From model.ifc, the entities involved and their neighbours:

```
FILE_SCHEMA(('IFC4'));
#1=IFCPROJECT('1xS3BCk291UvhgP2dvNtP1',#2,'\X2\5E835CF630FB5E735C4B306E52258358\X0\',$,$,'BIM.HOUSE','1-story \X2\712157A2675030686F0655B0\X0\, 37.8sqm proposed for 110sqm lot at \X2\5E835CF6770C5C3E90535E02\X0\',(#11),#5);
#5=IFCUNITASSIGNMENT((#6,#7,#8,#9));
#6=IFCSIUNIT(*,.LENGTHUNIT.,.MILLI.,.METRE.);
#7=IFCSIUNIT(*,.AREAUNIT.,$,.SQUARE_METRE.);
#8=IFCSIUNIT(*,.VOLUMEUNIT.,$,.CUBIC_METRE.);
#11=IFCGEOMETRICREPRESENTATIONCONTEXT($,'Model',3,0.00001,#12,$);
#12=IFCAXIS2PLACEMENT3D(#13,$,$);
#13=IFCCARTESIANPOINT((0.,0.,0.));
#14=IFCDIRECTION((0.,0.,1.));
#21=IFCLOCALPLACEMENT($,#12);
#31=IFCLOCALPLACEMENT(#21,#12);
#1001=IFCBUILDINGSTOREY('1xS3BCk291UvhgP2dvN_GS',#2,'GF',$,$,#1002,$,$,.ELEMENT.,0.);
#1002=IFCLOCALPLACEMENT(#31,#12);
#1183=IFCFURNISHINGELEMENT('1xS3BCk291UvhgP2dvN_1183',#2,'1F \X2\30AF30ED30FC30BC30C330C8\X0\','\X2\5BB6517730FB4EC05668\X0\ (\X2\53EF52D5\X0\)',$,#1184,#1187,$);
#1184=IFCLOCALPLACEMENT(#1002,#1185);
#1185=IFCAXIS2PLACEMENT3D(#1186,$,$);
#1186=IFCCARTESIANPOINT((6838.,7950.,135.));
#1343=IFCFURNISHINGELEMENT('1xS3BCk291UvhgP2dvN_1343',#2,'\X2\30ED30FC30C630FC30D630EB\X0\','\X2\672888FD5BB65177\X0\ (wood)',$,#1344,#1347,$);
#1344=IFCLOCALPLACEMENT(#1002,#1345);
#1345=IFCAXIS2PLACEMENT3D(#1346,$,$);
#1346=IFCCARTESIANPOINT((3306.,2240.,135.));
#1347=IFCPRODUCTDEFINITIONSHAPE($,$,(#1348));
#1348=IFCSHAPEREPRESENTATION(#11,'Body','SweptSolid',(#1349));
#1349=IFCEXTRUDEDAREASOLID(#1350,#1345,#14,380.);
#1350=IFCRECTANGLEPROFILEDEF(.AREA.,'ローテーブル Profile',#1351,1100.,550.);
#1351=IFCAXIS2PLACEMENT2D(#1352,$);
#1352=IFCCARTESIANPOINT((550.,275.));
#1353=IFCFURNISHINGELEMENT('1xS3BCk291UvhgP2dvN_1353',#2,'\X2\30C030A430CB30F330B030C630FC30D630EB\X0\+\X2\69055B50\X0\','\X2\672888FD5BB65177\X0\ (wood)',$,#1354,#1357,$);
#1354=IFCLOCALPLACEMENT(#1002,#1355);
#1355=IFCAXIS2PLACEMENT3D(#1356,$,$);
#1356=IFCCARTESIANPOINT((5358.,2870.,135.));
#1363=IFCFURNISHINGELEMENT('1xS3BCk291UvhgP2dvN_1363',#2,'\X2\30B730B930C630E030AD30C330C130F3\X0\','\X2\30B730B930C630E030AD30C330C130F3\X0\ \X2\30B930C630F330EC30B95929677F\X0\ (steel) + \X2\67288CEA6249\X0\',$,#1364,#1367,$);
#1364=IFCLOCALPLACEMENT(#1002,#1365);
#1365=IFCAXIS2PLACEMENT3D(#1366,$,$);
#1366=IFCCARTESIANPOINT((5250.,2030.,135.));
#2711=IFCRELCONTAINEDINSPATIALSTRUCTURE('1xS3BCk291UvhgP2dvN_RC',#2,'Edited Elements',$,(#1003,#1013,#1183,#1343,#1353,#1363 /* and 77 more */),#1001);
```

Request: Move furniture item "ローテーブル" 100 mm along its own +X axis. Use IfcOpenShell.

```python
import ifcopenshell
import ifcopenshell.api.geometry
import ifcopenshell.util.placement

model = ifcopenshell.open("model.ifc")

item = model.by_guid("1xS3BCk291UvhgP2dvN_1343")
matrix = ifcopenshell.util.placement.get_local_placement(item.ObjectPlacement)
matrix[:3, 3] += matrix[:3, 0] * 100.0
ifcopenshell.api.geometry.edit_object_placement(model, product=item, matrix=matrix, is_si=False)

print(ifcopenshell.util.placement.get_local_placement(item.ObjectPlacement).round(3) + 0.0)

model.write("model_rev.ifc")
```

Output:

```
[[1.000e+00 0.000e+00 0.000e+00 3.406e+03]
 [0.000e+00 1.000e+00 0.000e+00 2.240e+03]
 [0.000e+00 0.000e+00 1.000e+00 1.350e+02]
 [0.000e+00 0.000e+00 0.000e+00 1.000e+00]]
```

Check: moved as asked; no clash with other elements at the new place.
